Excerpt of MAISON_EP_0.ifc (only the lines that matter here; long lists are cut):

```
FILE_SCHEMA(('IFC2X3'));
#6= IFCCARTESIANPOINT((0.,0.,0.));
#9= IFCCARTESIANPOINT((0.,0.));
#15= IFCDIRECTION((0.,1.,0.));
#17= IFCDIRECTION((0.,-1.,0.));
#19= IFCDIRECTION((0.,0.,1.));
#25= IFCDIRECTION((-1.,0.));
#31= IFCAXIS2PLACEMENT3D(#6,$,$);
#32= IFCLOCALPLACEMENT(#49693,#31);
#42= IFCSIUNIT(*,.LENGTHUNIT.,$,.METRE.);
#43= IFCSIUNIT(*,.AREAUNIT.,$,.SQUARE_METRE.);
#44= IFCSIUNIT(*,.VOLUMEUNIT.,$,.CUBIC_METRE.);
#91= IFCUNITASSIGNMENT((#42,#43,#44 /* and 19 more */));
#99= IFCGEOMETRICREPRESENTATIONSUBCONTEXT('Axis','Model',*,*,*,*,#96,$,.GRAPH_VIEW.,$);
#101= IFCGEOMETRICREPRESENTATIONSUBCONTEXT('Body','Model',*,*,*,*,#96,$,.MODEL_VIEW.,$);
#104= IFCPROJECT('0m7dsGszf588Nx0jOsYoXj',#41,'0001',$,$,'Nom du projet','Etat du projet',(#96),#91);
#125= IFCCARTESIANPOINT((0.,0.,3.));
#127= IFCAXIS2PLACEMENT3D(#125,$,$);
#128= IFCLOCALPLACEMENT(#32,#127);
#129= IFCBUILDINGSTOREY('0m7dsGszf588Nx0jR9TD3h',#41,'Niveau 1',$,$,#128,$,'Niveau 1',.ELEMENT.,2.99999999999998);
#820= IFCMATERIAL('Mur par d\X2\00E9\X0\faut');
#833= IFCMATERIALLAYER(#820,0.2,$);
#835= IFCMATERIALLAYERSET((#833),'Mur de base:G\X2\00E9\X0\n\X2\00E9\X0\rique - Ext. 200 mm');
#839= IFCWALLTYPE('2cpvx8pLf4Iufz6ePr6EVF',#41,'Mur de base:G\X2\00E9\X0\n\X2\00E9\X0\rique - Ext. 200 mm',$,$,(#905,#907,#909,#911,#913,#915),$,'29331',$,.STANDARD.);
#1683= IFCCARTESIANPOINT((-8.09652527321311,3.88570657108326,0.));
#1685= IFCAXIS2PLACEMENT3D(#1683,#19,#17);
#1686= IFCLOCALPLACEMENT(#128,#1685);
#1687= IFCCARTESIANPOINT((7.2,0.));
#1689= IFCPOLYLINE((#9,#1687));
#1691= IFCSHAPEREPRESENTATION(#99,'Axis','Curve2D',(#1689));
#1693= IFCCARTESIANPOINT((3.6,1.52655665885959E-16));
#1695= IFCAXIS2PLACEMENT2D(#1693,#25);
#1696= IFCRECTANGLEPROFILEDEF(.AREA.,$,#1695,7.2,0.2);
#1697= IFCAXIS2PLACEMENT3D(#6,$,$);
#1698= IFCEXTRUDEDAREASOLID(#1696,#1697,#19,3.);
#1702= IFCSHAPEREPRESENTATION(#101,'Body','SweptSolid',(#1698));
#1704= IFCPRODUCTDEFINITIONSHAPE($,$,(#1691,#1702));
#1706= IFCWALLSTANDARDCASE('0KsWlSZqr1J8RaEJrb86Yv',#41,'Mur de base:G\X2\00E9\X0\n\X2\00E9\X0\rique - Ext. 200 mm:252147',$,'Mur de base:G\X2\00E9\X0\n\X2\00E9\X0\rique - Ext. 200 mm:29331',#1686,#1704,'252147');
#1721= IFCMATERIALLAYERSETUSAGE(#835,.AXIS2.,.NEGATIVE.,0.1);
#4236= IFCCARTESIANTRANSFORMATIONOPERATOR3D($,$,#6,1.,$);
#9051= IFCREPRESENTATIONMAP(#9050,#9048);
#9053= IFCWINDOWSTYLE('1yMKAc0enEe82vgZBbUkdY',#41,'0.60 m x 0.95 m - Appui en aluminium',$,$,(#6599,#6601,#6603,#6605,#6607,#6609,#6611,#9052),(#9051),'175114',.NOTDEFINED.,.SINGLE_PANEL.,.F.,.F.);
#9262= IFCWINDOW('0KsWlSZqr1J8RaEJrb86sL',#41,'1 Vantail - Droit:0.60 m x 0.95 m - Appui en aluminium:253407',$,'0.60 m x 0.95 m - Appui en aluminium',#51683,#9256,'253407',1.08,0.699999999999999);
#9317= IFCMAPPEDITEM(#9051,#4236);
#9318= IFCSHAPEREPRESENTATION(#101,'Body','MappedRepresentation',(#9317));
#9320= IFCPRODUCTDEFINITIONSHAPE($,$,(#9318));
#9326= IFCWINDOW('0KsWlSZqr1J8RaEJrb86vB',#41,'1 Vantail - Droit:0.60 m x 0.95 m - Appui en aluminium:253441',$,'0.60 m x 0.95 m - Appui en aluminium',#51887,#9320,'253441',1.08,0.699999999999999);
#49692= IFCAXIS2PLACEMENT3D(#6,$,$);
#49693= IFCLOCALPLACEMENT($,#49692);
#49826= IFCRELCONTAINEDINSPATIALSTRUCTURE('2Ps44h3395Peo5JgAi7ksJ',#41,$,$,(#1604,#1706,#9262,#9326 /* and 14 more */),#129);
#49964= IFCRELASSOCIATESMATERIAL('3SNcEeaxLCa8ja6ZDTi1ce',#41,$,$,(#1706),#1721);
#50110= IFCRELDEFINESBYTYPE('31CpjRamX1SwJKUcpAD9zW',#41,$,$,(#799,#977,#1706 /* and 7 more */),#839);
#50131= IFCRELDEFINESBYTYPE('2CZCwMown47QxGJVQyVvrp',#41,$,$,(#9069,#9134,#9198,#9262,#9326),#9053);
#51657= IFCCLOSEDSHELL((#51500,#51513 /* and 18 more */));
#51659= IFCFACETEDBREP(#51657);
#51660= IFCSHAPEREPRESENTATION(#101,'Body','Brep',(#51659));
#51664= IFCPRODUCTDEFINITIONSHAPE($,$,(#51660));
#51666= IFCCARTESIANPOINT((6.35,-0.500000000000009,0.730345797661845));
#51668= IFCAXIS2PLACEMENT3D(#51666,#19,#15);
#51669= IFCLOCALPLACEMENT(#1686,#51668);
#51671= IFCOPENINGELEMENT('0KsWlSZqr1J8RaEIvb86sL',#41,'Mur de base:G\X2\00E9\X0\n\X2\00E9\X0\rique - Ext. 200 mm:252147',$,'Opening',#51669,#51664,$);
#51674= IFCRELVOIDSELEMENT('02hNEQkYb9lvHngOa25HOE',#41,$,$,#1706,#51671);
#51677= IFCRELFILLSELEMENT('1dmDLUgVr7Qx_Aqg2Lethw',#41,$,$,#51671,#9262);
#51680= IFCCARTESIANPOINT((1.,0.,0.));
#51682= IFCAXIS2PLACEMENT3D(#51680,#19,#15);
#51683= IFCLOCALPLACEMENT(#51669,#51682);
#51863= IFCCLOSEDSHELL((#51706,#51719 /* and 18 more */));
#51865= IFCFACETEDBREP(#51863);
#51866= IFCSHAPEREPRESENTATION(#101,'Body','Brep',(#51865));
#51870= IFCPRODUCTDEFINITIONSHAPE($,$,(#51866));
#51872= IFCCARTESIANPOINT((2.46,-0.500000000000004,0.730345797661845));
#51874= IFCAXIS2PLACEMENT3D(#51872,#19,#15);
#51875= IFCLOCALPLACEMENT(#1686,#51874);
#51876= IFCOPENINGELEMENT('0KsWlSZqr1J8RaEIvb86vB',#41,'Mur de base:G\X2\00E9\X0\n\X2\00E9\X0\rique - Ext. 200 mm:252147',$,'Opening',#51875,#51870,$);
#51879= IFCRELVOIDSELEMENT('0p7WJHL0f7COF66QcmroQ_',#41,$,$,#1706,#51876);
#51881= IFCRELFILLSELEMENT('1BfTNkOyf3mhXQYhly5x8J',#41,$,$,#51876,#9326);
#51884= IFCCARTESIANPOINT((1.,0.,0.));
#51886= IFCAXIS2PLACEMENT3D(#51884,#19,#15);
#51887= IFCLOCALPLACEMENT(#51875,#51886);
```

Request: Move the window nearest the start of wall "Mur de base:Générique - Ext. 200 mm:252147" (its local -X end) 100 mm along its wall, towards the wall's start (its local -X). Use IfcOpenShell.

```python
import ifcopenshell
import ifcopenshell.api.geometry
import ifcopenshell.util.placement
import ifcopenshell.util.unit

model = ifcopenshell.open("MAISON_EP_0.ifc")
unit_scale = ifcopenshell.util.unit.calculate_unit_scale(model)

window = model.by_guid("0KsWlSZqr1J8RaEJrb86vB")
opening = window.FillsVoids[0].RelatingOpeningElement
wall = opening.VoidsElements[0].RelatingBuildingElement

wall_matrix = ifcopenshell.util.placement.get_local_placement(wall.ObjectPlacement)
shift = wall_matrix[:3, 0] * -0.1 / unit_scale
before = ifcopenshell.util.placement.get_local_placement(window.ObjectPlacement)[:3, 3].copy()

# The window is placed relative to its opening, so it follows when the opening moves.
matrix = ifcopenshell.util.placement.get_local_placement(opening.ObjectPlacement)
matrix[:3, 3] += shift
ifcopenshell.api.geometry.edit_object_placement(
    model, product=opening, matrix=matrix, is_si=False, should_transform_children=True
)

after = ifcopenshell.util.placement.get_local_placement(window.ObjectPlacement)[:3, 3]
print("window moved by", (after - before).round(3) + 0.0)

model.write("MAISON_EP_0-out.ifc")
```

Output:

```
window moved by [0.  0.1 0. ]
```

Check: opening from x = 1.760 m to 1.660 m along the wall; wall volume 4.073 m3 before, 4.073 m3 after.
